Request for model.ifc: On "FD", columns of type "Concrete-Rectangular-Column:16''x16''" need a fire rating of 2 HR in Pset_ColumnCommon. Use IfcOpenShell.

First a look at what the model holds.

```python
import ifcopenshell
import ifcopenshell.util.element

model = ifcopenshell.open("model.ifc")
print(model.schema)
storey = next(s for s in model.by_type("IfcBuildingStorey") if s.Name == "FD")
columns = [e for e in ifcopenshell.util.element.get_decomposition(storey) if e.is_a("IfcColumn")]
seen = {}
for e in columns:
    element_type = ifcopenshell.util.element.get_type(e)
    key = (element_type.Name if element_type != e and element_type else None, ifcopenshell.util.element.get_pset(e, "Pset_ColumnCommon", "FireRating"))
    seen[key] = seen.get(key, 0) + 1
for (name, value), count in sorted(seen.items(), key=str):
    print(count, "x", name, "|", value)
```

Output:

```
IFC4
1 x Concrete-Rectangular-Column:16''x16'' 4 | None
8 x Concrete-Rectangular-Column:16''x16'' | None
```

```python
import ifcopenshell
import ifcopenshell.api.pset
import ifcopenshell.util.element

model = ifcopenshell.open("model.ifc")

storey = next(s for s in model.by_type("IfcBuildingStorey") if s.Name == "FD")
columns = [e for e in ifcopenshell.util.element.get_decomposition(storey) if e.is_a("IfcColumn")]

count = 0
for e in columns:
    element_type = ifcopenshell.util.element.get_type(e)
    if element_type in (None, e) or element_type.Name != "Concrete-Rectangular-Column:16''x16''":
        continue
    # add_pset returns the element's existing set when there is one.
    pset = ifcopenshell.api.pset.add_pset(model, product=e, name="Pset_ColumnCommon")
    ifcopenshell.api.pset.edit_pset(model, pset=pset, properties={"FireRating": "2 HR"})
    count += 1

print(count, "columns updated")

model.write("model_v2.ifc")
```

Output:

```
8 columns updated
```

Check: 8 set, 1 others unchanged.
